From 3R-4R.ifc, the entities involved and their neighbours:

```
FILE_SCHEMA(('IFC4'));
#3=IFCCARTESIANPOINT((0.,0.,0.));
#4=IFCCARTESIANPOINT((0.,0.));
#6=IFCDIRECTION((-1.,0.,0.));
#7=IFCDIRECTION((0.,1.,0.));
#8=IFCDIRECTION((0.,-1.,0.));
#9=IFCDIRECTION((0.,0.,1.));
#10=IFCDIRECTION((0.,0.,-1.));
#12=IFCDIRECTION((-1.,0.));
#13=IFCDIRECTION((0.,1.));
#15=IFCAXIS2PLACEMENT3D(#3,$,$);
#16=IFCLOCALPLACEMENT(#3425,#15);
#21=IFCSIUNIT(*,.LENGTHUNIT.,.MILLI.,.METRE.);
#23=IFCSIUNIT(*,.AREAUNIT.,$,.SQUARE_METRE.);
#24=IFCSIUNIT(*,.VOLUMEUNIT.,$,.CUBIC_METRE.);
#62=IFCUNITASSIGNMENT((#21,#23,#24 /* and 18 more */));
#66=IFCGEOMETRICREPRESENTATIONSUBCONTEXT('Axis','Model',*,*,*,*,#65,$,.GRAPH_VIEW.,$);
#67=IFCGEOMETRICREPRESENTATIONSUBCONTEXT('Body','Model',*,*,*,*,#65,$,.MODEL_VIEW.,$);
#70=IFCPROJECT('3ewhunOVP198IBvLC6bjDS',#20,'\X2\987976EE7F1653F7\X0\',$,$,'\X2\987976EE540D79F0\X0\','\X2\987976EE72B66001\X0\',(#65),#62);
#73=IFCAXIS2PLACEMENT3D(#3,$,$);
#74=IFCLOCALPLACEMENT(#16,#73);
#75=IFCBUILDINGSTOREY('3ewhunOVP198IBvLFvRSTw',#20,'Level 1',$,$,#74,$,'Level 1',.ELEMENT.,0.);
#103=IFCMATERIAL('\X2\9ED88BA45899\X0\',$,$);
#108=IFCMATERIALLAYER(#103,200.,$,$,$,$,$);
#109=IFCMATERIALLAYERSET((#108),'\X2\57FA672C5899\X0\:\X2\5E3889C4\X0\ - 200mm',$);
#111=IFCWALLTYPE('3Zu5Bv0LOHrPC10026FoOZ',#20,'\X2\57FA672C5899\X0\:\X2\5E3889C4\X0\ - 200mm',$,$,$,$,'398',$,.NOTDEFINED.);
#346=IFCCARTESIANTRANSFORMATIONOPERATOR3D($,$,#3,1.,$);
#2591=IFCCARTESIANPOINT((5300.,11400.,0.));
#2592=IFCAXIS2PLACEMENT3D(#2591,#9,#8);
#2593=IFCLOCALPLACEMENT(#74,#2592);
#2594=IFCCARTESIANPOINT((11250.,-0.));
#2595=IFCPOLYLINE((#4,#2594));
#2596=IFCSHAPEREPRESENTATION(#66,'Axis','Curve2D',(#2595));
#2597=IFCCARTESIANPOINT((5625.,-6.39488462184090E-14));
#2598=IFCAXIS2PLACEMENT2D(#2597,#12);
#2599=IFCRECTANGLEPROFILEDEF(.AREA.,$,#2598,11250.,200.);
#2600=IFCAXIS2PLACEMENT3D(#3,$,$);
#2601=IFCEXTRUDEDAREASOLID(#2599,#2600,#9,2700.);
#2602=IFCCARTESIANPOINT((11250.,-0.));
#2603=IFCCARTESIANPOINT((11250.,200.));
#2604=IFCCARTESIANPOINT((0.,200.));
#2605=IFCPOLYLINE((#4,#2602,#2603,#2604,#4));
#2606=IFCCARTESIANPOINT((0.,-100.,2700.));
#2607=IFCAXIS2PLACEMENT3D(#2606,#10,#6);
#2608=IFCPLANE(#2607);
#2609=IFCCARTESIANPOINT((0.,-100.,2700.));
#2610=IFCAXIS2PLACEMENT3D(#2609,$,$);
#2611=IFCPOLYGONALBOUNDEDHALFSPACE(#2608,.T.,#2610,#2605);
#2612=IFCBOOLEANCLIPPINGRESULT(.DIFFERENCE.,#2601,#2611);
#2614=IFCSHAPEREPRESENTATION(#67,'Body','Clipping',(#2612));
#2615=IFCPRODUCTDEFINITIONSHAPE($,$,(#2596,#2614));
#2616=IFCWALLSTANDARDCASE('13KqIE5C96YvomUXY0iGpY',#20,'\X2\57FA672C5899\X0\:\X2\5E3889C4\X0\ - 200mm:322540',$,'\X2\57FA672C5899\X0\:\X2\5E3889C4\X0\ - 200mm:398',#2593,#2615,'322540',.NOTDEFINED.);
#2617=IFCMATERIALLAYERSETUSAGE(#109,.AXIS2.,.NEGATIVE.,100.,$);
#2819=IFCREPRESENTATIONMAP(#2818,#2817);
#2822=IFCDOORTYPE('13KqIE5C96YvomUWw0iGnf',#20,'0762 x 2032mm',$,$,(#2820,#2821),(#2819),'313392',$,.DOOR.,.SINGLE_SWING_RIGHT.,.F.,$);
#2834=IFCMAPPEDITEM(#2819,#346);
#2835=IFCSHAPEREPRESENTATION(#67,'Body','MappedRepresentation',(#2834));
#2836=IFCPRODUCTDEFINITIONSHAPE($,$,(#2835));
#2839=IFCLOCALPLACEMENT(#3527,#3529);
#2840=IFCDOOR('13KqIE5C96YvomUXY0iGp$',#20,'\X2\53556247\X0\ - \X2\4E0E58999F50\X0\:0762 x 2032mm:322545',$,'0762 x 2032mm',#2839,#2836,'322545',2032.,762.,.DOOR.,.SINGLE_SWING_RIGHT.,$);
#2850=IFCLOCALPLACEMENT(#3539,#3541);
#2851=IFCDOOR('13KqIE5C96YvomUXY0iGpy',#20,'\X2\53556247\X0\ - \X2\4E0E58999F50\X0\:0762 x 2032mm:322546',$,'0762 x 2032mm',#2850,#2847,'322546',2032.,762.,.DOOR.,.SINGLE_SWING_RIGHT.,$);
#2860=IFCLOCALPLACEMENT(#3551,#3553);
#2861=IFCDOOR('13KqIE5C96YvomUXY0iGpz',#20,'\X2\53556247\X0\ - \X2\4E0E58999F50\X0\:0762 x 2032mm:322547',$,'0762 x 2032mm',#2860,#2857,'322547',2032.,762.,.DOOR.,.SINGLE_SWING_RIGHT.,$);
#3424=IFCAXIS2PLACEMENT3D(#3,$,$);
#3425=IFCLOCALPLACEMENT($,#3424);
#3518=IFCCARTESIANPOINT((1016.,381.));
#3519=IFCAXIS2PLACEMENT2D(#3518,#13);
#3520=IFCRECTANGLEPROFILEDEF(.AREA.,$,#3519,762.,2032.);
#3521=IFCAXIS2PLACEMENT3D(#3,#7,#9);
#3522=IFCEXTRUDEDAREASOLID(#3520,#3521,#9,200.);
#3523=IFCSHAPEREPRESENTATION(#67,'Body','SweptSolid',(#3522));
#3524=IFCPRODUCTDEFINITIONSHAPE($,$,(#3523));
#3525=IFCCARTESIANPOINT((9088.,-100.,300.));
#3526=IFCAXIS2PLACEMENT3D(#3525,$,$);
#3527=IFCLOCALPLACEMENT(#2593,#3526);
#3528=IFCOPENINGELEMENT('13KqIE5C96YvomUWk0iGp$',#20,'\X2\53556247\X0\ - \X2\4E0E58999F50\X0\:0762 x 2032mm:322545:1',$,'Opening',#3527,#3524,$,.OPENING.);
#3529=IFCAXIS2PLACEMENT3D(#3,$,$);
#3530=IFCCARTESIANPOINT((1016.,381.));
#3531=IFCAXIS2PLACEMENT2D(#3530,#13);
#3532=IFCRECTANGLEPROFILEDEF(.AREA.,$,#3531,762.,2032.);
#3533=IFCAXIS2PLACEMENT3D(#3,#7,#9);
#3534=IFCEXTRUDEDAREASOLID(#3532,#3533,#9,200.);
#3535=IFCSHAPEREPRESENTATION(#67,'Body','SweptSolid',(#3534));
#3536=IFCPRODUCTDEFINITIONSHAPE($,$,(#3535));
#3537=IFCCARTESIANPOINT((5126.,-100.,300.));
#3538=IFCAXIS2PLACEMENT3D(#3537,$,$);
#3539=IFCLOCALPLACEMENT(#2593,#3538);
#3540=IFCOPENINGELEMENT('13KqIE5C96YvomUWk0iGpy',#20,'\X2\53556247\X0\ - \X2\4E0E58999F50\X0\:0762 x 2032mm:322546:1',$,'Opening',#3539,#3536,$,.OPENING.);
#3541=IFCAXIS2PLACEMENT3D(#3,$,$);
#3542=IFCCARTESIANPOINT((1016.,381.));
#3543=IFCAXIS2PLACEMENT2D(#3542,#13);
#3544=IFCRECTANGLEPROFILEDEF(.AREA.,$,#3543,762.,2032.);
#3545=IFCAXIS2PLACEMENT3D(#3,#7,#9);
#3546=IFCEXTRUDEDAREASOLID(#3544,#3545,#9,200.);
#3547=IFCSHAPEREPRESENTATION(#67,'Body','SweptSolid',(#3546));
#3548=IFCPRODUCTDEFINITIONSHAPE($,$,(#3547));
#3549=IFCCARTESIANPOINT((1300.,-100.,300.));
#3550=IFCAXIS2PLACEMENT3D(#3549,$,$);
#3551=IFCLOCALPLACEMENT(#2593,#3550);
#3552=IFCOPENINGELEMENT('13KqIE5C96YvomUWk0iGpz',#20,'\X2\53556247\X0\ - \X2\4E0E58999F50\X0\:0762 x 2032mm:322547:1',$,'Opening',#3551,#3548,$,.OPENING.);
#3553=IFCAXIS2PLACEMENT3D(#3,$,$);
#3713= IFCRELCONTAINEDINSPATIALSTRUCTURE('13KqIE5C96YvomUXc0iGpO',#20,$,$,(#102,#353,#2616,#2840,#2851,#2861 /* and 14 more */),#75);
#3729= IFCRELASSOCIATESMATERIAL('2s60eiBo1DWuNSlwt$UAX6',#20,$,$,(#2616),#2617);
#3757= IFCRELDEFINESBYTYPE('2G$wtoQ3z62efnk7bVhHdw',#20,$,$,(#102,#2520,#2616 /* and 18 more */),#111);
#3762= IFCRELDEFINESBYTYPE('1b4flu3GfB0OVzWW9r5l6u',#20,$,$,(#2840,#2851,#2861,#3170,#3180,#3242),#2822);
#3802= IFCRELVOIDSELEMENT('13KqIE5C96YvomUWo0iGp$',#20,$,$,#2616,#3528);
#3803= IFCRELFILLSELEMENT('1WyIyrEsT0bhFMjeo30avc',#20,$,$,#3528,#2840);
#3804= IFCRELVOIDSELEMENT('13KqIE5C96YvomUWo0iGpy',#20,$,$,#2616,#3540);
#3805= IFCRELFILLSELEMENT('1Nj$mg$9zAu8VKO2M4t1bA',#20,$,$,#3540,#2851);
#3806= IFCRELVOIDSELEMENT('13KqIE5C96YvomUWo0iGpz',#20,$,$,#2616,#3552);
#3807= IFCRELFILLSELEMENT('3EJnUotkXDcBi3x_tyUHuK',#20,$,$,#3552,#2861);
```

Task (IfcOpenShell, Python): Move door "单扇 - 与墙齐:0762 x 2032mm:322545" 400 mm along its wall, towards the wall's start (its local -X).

```python
import ifcopenshell
import ifcopenshell.api.geometry
import ifcopenshell.util.placement
import ifcopenshell.util.unit

model = ifcopenshell.open("3R-4R.ifc")
unit_scale = ifcopenshell.util.unit.calculate_unit_scale(model)

door = model.by_guid("13KqIE5C96YvomUXY0iGp$")
opening = door.FillsVoids[0].RelatingOpeningElement
wall = opening.VoidsElements[0].RelatingBuildingElement

wall_matrix = ifcopenshell.util.placement.get_local_placement(wall.ObjectPlacement)
shift = wall_matrix[:3, 0] * -0.4 / unit_scale
before = ifcopenshell.util.placement.get_local_placement(door.ObjectPlacement)[:3, 3].copy()

# The door is placed relative to its opening, so it follows when the opening moves.
matrix = ifcopenshell.util.placement.get_local_placement(opening.ObjectPlacement)
matrix[:3, 3] += shift
ifcopenshell.api.geometry.edit_object_placement(
    model, product=opening, matrix=matrix, is_si=False, should_transform_children=True
)

after = ifcopenshell.util.placement.get_local_placement(door.ObjectPlacement)[:3, 3]
print("door moved by", (after - before).round(3) + 0.0)

model.write("3R-4R_v2.ifc")
```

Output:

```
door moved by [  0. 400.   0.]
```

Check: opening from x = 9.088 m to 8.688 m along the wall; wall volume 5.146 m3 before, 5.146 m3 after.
